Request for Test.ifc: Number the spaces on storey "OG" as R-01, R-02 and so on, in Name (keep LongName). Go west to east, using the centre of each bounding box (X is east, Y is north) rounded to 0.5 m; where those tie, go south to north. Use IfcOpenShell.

First a look at what the model holds.

```python
import ifcopenshell
import ifcopenshell.util.element
import ifcopenshell.util.placement

model = ifcopenshell.open("Test.ifc")
print(model.schema)
storey = next(s for s in model.by_type("IfcBuildingStorey") if s.Name == "OG")
spaces = [e for e in ifcopenshell.util.element.get_decomposition(storey) if e.is_a("IfcSpace")]
for e in sorted(spaces, key=lambda e: e.id()):
    origin = ifcopenshell.util.placement.get_local_placement(e.ObjectPlacement)[:3, 3]
    print(e.id(), e.Name, e.LongName, origin.round(2) + 0.0, sep=" | ")
```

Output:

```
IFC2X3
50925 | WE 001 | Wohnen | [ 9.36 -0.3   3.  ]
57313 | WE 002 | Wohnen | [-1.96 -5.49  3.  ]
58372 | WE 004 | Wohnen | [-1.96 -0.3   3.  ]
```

```python
import ifcopenshell
import ifcopenshell.geom
import ifcopenshell.util.element
import ifcopenshell.util.shape

model = ifcopenshell.open("Test.ifc")
settings = ifcopenshell.geom.settings()
settings.set("use-world-coords", True)


def centre(element):
    shape = ifcopenshell.geom.create_shape(settings, element)
    return ifcopenshell.util.shape.get_bbox_centroid(shape.geometry)


storey = next(s for s in model.by_type("IfcBuildingStorey") if s.Name == "OG")
spaces = [e for e in ifcopenshell.util.element.get_decomposition(storey) if e.is_a("IfcSpace")]

# Insertion points can sit at a corner or the storey origin, so sort by the geometry (in metres).
centres = {e: centre(e) for e in spaces}
spaces.sort(key=lambda e: (round(centres[e][0] / 0.5), centres[e][1]))

for i, e in enumerate(spaces, start=1):
    number = f"R-{i:02d}"
    e.Name = number
    print(e.id(), number)

model.write("Test_edited.ifc")
```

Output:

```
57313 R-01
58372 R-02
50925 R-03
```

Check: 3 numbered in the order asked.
